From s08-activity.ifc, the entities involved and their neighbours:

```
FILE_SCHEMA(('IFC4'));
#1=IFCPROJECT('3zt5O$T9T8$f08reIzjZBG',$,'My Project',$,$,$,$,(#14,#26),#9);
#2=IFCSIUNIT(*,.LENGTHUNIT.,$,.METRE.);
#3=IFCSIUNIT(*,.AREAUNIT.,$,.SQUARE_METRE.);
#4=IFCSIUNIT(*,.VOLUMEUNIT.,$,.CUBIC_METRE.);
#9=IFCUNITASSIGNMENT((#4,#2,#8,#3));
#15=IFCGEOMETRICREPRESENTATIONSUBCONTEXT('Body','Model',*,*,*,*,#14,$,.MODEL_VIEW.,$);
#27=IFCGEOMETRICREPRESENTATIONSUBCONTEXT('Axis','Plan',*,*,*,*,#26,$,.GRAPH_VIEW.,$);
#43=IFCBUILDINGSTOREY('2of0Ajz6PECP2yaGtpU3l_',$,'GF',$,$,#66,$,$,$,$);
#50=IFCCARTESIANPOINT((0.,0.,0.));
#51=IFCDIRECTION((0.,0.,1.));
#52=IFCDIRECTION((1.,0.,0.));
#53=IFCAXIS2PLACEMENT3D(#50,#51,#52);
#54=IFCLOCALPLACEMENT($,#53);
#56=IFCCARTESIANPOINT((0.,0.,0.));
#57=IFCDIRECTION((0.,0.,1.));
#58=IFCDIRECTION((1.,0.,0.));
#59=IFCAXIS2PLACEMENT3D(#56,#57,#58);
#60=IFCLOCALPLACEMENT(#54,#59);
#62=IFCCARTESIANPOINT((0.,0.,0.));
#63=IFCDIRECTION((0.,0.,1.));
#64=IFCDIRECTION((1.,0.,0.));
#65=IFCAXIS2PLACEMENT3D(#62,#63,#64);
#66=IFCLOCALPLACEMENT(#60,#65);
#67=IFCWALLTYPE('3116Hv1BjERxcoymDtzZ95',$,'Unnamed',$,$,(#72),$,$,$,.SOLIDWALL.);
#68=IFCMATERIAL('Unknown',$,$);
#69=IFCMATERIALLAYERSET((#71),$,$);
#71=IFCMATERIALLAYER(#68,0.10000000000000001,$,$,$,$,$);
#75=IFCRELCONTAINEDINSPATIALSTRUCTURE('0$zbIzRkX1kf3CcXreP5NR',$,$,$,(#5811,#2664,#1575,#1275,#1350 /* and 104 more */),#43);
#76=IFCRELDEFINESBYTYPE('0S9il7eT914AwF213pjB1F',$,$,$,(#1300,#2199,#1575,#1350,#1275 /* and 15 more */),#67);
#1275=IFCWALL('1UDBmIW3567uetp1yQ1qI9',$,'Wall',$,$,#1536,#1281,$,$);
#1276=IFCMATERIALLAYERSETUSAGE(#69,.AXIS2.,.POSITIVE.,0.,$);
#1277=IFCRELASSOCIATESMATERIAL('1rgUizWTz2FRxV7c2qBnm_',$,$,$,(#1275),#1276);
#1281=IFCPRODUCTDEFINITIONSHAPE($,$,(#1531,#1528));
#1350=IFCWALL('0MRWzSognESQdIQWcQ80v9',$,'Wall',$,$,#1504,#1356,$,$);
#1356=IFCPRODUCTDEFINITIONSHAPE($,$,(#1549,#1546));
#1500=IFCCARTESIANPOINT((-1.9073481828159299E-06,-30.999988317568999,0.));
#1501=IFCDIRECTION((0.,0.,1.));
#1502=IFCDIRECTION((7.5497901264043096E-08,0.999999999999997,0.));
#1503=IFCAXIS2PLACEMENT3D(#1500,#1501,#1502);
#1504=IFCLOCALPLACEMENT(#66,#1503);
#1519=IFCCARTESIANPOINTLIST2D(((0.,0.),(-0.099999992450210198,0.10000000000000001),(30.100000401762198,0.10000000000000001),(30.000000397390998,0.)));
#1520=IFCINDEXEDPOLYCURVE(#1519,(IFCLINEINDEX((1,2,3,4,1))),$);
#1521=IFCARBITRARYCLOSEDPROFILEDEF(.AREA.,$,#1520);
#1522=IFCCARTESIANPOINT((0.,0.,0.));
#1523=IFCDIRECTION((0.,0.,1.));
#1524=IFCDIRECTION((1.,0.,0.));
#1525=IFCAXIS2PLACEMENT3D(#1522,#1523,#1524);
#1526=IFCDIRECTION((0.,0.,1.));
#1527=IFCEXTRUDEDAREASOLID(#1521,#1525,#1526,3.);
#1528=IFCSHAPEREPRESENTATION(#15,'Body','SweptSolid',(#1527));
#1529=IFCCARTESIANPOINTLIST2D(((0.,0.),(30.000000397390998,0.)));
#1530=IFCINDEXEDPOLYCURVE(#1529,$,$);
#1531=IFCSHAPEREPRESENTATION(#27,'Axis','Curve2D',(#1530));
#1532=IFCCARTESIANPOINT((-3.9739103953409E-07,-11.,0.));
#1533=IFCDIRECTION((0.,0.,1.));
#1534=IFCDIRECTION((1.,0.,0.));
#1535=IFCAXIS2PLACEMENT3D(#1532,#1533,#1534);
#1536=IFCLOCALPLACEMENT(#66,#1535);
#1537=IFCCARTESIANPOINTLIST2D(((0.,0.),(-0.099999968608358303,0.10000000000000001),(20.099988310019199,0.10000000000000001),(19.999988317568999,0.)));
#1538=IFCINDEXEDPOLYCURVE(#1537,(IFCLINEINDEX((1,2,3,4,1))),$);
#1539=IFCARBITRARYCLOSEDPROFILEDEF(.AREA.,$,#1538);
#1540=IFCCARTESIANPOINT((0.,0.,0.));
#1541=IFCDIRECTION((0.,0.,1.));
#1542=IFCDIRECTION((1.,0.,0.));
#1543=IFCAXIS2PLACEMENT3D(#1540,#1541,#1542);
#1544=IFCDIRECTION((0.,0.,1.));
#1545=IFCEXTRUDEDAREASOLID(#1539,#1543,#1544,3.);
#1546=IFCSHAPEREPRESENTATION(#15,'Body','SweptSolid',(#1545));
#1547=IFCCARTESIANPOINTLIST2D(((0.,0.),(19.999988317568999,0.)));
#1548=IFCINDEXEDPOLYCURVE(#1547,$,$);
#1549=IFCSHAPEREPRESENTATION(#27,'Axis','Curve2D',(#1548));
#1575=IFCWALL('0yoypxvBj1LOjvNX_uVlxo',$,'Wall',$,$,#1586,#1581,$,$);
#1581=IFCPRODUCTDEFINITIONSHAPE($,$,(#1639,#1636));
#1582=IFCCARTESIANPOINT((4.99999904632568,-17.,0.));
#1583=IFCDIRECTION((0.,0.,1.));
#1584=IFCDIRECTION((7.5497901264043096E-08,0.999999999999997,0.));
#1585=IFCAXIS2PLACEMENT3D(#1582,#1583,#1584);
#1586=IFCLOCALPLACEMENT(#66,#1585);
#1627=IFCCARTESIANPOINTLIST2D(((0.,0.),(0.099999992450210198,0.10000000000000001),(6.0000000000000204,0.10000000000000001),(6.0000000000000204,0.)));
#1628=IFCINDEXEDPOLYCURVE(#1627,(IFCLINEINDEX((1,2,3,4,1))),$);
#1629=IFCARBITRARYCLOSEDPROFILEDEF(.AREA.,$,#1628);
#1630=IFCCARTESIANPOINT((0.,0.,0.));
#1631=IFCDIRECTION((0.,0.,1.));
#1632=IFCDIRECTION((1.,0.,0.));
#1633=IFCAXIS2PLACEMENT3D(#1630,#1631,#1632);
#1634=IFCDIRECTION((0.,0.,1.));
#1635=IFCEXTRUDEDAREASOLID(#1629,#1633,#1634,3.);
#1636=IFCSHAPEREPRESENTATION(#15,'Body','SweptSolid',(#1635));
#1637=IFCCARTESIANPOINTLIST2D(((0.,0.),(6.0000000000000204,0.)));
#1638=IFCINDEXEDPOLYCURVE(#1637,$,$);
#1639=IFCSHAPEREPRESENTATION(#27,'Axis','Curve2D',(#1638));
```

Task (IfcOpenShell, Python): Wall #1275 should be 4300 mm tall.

```python
import ifcopenshell
import ifcopenshell.geom
import ifcopenshell.util.representation
import ifcopenshell.util.shape
import ifcopenshell.util.unit

model = ifcopenshell.open("s08-activity.ifc")
unit_scale = ifcopenshell.util.unit.calculate_unit_scale(model)
settings = ifcopenshell.geom.settings()


def volume(element):
    """Net volume in cubic metres, openings subtracted."""
    shape = ifcopenshell.geom.create_shape(settings, element)
    return ifcopenshell.util.shape.get_volume(shape.geometry)


wall = model.by_id(1275)
before = volume(wall)

body = ifcopenshell.util.representation.get_representation(wall, "Model", "Body")
solid = body.Items[0]
old_height = solid.Depth
solid.Depth = 4.3 / unit_scale
after = volume(wall)

print(f"height {old_height:g} -> {solid.Depth:g}, volume {before:.3f} -> {after:.3f} m3")

model.write("s08-activity_edited.ifc")
```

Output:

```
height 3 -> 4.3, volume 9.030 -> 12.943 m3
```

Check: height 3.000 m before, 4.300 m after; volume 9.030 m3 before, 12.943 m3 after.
